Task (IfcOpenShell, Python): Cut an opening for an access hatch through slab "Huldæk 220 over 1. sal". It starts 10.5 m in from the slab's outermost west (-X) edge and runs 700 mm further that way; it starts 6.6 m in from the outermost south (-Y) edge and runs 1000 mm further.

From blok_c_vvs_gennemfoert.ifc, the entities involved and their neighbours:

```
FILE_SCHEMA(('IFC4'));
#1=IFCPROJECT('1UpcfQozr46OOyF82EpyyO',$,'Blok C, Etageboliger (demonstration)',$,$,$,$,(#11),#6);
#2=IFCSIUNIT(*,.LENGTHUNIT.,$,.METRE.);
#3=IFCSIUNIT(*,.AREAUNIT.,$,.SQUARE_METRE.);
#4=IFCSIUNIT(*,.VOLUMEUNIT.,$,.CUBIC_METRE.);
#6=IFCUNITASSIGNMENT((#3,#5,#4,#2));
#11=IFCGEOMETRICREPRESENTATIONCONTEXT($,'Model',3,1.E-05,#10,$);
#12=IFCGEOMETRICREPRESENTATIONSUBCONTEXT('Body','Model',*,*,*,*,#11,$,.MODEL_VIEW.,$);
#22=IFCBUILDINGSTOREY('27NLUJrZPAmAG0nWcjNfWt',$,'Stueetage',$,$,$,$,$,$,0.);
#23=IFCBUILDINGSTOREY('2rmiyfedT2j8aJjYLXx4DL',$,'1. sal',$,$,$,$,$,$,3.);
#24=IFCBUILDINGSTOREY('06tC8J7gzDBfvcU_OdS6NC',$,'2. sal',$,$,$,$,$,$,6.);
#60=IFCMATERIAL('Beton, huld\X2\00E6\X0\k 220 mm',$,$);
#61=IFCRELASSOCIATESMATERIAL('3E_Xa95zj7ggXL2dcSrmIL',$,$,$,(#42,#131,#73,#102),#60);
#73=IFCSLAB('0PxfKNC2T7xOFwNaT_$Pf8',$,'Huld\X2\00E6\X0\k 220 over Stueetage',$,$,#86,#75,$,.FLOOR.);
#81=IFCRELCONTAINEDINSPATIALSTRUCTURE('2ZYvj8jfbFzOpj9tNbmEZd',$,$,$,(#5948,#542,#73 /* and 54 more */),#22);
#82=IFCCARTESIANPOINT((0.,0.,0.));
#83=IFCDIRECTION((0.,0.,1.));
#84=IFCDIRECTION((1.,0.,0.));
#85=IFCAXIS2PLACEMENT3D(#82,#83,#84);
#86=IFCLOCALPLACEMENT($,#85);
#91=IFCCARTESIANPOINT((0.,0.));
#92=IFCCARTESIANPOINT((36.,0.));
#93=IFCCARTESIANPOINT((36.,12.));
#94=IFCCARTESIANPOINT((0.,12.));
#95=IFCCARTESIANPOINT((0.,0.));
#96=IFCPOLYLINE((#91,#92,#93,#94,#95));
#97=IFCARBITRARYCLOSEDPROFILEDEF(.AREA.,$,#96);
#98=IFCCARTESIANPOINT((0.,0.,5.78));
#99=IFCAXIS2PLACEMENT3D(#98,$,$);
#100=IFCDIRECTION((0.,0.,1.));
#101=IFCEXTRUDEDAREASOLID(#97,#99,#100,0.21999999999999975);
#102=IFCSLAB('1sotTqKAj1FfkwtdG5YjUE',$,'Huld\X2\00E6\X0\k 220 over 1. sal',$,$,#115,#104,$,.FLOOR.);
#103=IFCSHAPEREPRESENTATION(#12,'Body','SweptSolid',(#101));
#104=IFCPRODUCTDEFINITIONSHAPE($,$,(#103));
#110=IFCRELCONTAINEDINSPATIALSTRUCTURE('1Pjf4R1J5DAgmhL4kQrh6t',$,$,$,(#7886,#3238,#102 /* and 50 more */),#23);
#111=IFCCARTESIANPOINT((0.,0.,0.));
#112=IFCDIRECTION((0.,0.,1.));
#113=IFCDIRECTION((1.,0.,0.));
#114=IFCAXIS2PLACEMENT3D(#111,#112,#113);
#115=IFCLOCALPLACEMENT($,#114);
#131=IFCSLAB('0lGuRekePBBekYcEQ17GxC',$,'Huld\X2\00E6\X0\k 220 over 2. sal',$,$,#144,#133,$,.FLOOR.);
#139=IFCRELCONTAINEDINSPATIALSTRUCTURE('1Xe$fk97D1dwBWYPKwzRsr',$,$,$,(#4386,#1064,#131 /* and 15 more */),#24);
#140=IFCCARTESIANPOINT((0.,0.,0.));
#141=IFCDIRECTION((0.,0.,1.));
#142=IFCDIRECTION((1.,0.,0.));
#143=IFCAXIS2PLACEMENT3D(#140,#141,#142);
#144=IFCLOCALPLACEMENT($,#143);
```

```python
import numpy as np
import ifcopenshell
import ifcopenshell.api.feature
import ifcopenshell.api.geometry
import ifcopenshell.api.root
import ifcopenshell.geom
import ifcopenshell.util.placement
import ifcopenshell.util.representation
import ifcopenshell.util.shape
import ifcopenshell.util.unit

model = ifcopenshell.open("blok_c_vvs_gennemfoert.ifc")
unit_scale = ifcopenshell.util.unit.calculate_unit_scale(model)
settings = ifcopenshell.geom.settings()


def volume(element):
    """Net volume in cubic metres, openings subtracted."""
    shape = ifcopenshell.geom.create_shape(settings, element)
    return ifcopenshell.util.shape.get_volume(shape.geometry)


slab = model.by_id(102)
before = volume(slab)

# Extent in the slab's own axes, in metres. The edges named are its -X and -Y sides.
slab_shape = ifcopenshell.geom.create_shape(settings, slab)
vertices = ifcopenshell.util.shape.get_vertices(slab_shape.geometry)
x_min, y_min, bottom = vertices.min(axis=0)
top = vertices[:, 2].max()

opening = ifcopenshell.api.root.create_entity(model, ifc_class="IfcOpeningElement", name="Access hatch opening", predefined_type="OPENING")
context = ifcopenshell.util.representation.get_context(model, "Model", "Body", "MODEL_VIEW")
width, depth = 0.7, 1
outline = [(0.0, 0.0), (width, 0.0), (width, depth), (0.0, depth), (0.0, 0.0)]
# Overshoot both faces by 50 mm so the cut is clean.
shape = ifcopenshell.api.geometry.add_slab_representation(
    model, context=context, depth=top - bottom + 0.1, polyline=outline
)
ifcopenshell.api.geometry.assign_representation(model, product=opening, representation=shape)

matrix = ifcopenshell.util.placement.get_local_placement(slab.ObjectPlacement)
matrix[:, 3] = matrix @ np.append(np.array([x_min + 10.5, y_min + 6.6, bottom - 0.05]) / unit_scale, 1.0)
ifcopenshell.api.geometry.edit_object_placement(model, product=opening, matrix=matrix, is_si=False)
ifcopenshell.api.feature.add_feature(model, feature=opening, element=slab)

after = volume(slab)

print(f"slab volume {before:.3f} -> {after:.3f} m3")

model.write("blok_c_vvs_gennemfoert_rev.ifc")
```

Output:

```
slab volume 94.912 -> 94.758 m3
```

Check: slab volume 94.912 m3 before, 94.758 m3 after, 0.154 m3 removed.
